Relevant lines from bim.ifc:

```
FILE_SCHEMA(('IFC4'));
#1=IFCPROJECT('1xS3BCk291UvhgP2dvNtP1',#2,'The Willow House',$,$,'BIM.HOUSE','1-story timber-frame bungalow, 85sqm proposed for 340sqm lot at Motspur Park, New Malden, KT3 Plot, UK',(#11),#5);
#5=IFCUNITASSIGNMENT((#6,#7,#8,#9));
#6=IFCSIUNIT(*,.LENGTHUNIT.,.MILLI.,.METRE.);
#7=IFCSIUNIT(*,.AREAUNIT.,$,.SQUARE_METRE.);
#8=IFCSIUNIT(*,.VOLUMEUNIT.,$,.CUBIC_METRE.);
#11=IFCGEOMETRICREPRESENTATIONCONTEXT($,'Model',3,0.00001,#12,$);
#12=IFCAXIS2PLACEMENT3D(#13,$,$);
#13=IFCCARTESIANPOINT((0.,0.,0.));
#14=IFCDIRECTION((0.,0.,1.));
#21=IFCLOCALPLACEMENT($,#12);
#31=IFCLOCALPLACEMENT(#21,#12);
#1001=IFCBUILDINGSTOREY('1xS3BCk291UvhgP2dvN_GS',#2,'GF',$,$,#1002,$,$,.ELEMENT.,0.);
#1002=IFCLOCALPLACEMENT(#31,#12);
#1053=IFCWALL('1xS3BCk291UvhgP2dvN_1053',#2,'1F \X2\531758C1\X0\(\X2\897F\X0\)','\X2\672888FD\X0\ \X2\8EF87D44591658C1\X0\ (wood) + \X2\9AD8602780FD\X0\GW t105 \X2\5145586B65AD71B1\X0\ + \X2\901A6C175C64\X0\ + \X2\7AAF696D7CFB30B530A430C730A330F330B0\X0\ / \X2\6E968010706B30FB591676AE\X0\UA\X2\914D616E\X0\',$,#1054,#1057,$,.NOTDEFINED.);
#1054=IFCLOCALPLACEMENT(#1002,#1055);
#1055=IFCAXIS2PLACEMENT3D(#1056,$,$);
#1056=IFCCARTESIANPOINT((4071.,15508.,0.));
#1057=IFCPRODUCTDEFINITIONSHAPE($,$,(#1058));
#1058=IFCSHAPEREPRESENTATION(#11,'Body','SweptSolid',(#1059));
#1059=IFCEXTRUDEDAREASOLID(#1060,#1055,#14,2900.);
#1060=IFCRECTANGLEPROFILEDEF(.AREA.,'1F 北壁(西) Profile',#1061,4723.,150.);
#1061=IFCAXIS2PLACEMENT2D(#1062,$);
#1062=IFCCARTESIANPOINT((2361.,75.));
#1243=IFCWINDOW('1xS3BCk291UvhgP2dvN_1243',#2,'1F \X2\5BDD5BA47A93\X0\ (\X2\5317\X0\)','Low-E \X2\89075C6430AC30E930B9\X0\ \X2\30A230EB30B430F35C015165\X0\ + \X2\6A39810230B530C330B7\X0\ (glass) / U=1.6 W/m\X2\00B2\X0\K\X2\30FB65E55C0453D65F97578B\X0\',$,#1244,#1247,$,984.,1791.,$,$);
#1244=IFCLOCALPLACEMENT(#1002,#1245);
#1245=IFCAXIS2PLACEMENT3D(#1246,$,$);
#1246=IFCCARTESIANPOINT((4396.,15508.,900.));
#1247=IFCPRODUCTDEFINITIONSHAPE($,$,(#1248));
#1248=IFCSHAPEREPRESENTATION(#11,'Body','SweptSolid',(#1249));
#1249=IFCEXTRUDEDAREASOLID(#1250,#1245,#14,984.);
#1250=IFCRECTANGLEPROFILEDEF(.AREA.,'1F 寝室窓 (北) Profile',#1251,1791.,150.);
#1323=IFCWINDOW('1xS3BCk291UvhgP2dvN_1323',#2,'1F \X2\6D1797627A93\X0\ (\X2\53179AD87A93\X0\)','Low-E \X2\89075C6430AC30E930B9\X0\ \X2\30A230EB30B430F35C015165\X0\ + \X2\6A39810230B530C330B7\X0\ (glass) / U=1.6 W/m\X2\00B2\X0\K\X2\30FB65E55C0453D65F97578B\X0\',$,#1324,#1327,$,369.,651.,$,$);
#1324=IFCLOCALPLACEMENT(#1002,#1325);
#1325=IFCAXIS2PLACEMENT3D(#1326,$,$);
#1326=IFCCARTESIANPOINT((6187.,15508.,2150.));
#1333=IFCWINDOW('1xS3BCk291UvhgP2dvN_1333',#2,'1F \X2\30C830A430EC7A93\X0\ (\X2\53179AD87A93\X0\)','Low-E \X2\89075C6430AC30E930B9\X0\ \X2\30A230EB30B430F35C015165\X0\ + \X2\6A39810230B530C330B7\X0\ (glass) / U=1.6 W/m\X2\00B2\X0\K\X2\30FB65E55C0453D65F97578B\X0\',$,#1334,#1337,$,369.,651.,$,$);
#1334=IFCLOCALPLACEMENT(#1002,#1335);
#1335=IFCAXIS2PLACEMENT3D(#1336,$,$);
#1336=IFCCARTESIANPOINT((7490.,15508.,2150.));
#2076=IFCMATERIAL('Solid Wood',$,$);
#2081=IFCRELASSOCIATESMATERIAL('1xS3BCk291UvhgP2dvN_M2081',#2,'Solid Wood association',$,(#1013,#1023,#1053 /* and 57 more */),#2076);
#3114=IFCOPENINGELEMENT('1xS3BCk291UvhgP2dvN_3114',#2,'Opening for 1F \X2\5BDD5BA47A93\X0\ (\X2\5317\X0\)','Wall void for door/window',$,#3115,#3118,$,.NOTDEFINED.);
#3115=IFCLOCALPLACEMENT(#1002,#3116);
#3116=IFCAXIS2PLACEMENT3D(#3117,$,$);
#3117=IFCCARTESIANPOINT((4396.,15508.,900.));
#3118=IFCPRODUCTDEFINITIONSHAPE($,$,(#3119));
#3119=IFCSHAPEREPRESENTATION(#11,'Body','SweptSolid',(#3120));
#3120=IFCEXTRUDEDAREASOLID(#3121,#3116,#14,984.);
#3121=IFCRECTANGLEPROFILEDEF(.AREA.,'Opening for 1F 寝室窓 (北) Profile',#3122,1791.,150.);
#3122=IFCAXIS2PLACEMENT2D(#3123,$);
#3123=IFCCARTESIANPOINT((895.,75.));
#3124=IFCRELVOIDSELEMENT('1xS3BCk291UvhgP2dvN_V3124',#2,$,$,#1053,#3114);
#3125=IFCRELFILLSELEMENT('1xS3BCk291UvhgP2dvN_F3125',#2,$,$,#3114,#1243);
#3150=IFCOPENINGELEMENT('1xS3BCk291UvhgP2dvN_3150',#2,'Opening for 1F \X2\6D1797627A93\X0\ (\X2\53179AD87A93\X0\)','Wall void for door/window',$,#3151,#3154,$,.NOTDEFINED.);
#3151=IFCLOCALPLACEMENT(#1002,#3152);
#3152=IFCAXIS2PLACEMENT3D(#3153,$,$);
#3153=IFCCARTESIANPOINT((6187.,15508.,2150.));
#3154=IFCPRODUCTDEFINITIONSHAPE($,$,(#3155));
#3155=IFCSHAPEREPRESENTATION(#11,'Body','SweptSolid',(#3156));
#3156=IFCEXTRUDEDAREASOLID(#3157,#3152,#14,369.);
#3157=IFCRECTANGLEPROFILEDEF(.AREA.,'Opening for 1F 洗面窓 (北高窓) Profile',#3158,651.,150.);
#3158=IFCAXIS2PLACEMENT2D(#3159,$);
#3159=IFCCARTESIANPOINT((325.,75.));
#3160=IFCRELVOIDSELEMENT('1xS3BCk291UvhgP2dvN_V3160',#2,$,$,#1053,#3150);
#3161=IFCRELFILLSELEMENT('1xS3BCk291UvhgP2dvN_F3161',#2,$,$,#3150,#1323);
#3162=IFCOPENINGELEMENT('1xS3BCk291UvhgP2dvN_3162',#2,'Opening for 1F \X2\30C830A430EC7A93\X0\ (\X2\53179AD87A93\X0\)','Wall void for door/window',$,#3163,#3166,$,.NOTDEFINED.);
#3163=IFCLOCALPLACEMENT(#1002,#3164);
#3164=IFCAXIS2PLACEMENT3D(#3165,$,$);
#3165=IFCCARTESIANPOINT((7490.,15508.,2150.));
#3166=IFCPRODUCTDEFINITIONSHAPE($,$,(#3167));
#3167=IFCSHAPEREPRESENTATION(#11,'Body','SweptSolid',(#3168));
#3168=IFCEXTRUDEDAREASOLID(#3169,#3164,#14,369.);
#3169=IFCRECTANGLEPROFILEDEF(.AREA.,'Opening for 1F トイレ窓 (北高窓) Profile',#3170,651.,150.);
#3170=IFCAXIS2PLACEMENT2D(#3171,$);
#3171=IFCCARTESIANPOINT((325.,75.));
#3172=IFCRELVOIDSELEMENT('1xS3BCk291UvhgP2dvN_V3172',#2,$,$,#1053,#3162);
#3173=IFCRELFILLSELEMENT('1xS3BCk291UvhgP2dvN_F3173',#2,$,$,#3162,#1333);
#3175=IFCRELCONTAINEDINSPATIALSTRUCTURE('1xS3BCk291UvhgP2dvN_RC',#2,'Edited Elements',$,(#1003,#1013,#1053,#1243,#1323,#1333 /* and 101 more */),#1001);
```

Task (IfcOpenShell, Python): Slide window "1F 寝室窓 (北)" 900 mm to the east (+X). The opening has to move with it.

```python
import ifcopenshell
import ifcopenshell.api.geometry
import ifcopenshell.util.placement
import ifcopenshell.util.unit

model = ifcopenshell.open("bim.ifc")
unit_scale = ifcopenshell.util.unit.calculate_unit_scale(model)

window = model.by_guid("1xS3BCk291UvhgP2dvN_1243")
opening = window.FillsVoids[0].RelatingOpeningElement
wall = opening.VoidsElements[0].RelatingBuildingElement

wall_matrix = ifcopenshell.util.placement.get_local_placement(wall.ObjectPlacement)
shift = wall_matrix[:3, 0] * 0.9 / unit_scale
before = ifcopenshell.util.placement.get_local_placement(window.ObjectPlacement)[:3, 3].copy()

# The window is not placed relative to its opening, so move both.
for product in (opening, window):
    matrix = ifcopenshell.util.placement.get_local_placement(product.ObjectPlacement)
    matrix[:3, 3] += shift
    ifcopenshell.api.geometry.edit_object_placement(model, product=product, matrix=matrix, is_si=False)

after = ifcopenshell.util.placement.get_local_placement(window.ObjectPlacement)[:3, 3]
print("window moved by", (after - before).round(3) + 0.0)

model.write("bim_rev.ifc")
```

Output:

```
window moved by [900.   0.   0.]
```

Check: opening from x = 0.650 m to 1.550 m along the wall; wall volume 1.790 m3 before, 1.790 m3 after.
